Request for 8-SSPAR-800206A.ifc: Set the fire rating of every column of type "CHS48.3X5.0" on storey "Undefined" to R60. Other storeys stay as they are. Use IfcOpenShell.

First a look at what the model holds.

```python
import ifcopenshell
import ifcopenshell.util.element

model = ifcopenshell.open("8-SSPAR-800206A.ifc")
print(model.schema)
storey = next(s for s in model.by_type("IfcBuildingStorey") if s.Name == "Undefined")
columns = [e for e in ifcopenshell.util.element.get_decomposition(storey) if e.is_a("IfcColumn")]
seen = {}
for e in columns:
    element_type = ifcopenshell.util.element.get_type(e)
    key = (element_type.Name if element_type != e and element_type else None, ifcopenshell.util.element.get_pset(e, "Pset_ColumnCommon", "FireRating"))
    seen[key] = seen.get(key, 0) + 1
for (name, value), count in sorted(seen.items(), key=str):
    print(count, "x", name, "|", value)
```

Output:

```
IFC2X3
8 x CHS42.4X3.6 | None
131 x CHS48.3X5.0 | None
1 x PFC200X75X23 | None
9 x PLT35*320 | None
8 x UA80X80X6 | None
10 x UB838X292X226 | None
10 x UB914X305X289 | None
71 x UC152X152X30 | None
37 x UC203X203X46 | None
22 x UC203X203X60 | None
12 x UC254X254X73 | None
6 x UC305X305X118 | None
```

```python
import ifcopenshell
import ifcopenshell.api.pset
import ifcopenshell.util.element

model = ifcopenshell.open("8-SSPAR-800206A.ifc")

storey = next(s for s in model.by_type("IfcBuildingStorey") if s.Name == "Undefined")
columns = [e for e in ifcopenshell.util.element.get_decomposition(storey) if e.is_a("IfcColumn")]

count = 0
for e in columns:
    element_type = ifcopenshell.util.element.get_type(e)
    if element_type in (None, e) or element_type.Name != "CHS48.3X5.0":
        continue
    # add_pset returns the element's existing set when there is one.
    pset = ifcopenshell.api.pset.add_pset(model, product=e, name="Pset_ColumnCommon")
    ifcopenshell.api.pset.edit_pset(model, pset=pset, properties={"FireRating": "R60"})
    count += 1

print(count, "columns updated")

model.write("8-SSPAR-800206A_v2.ifc")
```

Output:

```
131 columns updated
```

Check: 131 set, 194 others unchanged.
